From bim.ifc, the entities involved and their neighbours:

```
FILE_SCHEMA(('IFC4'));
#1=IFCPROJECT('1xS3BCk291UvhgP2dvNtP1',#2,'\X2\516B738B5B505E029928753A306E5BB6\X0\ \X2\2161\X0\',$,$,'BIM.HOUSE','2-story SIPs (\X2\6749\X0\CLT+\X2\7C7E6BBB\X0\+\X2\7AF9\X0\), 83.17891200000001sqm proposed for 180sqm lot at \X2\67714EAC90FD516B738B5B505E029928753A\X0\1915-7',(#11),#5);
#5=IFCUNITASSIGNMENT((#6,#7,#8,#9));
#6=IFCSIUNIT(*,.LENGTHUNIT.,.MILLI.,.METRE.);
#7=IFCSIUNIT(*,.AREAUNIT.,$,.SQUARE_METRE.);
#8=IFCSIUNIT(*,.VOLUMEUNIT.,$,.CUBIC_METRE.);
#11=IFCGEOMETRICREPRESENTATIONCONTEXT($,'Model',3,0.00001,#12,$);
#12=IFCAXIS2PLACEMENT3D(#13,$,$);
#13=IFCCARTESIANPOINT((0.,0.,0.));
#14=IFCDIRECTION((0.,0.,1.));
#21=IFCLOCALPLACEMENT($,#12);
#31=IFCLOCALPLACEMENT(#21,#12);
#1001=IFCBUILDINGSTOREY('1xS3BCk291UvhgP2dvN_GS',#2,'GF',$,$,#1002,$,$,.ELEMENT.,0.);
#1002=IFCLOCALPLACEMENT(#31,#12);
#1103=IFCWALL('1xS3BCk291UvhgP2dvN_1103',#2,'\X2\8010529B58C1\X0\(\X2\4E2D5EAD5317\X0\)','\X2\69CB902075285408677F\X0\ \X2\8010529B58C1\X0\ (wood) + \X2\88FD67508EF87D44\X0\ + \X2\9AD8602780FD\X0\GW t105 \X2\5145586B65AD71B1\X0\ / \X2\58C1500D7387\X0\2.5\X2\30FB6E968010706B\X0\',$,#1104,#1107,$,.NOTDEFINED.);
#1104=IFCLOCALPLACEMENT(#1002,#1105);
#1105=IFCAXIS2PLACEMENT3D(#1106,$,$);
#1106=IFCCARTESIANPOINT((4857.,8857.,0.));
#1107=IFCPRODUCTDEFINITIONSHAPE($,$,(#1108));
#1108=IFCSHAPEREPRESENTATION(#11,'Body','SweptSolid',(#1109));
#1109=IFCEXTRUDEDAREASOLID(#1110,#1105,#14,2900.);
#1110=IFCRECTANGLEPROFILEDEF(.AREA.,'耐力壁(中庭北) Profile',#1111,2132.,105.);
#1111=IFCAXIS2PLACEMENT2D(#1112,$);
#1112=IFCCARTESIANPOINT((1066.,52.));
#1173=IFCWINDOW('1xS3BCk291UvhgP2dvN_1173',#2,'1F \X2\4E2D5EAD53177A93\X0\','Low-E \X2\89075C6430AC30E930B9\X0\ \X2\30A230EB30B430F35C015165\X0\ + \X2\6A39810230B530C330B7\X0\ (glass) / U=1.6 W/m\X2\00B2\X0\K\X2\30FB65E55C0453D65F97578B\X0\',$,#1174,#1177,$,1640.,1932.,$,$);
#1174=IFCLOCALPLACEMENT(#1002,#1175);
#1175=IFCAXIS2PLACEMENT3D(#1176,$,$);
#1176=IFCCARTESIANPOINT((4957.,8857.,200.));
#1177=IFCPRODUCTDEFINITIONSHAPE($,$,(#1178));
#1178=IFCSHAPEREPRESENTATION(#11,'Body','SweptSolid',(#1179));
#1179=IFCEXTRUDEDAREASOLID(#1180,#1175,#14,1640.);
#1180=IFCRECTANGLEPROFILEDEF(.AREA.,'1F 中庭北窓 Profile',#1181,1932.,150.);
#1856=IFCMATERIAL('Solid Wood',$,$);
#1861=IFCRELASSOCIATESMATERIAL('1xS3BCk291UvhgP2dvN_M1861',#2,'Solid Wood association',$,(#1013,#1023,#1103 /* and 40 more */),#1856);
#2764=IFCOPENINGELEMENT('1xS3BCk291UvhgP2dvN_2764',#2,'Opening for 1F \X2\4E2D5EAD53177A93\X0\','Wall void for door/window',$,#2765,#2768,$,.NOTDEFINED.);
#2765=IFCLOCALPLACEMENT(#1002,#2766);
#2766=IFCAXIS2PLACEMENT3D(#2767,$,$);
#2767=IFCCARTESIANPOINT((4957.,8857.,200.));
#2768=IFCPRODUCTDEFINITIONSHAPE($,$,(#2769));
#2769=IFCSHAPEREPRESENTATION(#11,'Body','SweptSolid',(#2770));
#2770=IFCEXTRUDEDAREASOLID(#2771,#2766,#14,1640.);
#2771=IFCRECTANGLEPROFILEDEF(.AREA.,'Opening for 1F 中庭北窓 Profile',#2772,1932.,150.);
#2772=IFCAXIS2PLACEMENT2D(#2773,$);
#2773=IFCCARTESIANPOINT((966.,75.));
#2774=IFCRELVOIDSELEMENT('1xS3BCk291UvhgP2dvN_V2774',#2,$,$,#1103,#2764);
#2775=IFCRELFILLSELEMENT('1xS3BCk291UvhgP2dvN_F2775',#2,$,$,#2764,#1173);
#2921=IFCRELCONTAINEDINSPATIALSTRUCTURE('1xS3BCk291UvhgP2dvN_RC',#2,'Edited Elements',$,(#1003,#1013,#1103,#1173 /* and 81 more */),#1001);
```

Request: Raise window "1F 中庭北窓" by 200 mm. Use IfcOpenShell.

```python
import numpy as np
import ifcopenshell
import ifcopenshell.api.geometry
import ifcopenshell.util.placement
import ifcopenshell.util.unit

model = ifcopenshell.open("bim.ifc")
unit_scale = ifcopenshell.util.unit.calculate_unit_scale(model)

window = model.by_guid("1xS3BCk291UvhgP2dvN_1173")
opening = window.FillsVoids[0].RelatingOpeningElement
dz = 200.0

shift = np.array([0.0, 0.0, dz])
# The window is not placed relative to its opening, so move both.
for product in (opening, window):
    matrix = ifcopenshell.util.placement.get_local_placement(product.ObjectPlacement)
    matrix[:3, 3] += shift
    ifcopenshell.api.geometry.edit_object_placement(model, product=product, matrix=matrix, is_si=False)

print(f"moved by {dz * unit_scale:+.3f} m")

model.write("bim_v2.ifc")
```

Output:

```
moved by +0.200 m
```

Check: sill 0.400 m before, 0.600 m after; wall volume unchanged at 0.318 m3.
